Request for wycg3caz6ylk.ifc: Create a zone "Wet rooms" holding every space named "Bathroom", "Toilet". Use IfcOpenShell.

First a look at what the model holds.

```python
import ifcopenshell

model = ifcopenshell.open("wycg3caz6ylk.ifc")
print(model.schema)
seen = {}
for space in model.by_type("IfcSpace"):
    seen[space.Name] = seen.get(space.Name, 0) + 1
for name, count in sorted(seen.items(), key=str):
    print(count, "x", name)
print("zones:", [z.Name for z in model.by_type("IfcZone")][:20])
```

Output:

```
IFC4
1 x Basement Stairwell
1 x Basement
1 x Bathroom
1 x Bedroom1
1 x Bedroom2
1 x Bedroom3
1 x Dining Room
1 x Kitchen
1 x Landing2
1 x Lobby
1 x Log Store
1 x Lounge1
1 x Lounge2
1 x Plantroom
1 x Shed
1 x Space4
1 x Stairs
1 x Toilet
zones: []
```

```python
import ifcopenshell
import ifcopenshell.api.group
import ifcopenshell.api.root

model = ifcopenshell.open("wycg3caz6ylk.ifc")

names = {"Bathroom", "Toilet"}
spaces = [s for s in model.by_type("IfcSpace") if s.Name in names]

zone = ifcopenshell.api.root.create_entity(model, ifc_class="IfcZone", name="Wet rooms")
ifcopenshell.api.group.assign_group(model, products=spaces, group=zone)
print(len(spaces), "spaces in", zone.Name)

model.write("wycg3caz6ylk_edited.ifc")
```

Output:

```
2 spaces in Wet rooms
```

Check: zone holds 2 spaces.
